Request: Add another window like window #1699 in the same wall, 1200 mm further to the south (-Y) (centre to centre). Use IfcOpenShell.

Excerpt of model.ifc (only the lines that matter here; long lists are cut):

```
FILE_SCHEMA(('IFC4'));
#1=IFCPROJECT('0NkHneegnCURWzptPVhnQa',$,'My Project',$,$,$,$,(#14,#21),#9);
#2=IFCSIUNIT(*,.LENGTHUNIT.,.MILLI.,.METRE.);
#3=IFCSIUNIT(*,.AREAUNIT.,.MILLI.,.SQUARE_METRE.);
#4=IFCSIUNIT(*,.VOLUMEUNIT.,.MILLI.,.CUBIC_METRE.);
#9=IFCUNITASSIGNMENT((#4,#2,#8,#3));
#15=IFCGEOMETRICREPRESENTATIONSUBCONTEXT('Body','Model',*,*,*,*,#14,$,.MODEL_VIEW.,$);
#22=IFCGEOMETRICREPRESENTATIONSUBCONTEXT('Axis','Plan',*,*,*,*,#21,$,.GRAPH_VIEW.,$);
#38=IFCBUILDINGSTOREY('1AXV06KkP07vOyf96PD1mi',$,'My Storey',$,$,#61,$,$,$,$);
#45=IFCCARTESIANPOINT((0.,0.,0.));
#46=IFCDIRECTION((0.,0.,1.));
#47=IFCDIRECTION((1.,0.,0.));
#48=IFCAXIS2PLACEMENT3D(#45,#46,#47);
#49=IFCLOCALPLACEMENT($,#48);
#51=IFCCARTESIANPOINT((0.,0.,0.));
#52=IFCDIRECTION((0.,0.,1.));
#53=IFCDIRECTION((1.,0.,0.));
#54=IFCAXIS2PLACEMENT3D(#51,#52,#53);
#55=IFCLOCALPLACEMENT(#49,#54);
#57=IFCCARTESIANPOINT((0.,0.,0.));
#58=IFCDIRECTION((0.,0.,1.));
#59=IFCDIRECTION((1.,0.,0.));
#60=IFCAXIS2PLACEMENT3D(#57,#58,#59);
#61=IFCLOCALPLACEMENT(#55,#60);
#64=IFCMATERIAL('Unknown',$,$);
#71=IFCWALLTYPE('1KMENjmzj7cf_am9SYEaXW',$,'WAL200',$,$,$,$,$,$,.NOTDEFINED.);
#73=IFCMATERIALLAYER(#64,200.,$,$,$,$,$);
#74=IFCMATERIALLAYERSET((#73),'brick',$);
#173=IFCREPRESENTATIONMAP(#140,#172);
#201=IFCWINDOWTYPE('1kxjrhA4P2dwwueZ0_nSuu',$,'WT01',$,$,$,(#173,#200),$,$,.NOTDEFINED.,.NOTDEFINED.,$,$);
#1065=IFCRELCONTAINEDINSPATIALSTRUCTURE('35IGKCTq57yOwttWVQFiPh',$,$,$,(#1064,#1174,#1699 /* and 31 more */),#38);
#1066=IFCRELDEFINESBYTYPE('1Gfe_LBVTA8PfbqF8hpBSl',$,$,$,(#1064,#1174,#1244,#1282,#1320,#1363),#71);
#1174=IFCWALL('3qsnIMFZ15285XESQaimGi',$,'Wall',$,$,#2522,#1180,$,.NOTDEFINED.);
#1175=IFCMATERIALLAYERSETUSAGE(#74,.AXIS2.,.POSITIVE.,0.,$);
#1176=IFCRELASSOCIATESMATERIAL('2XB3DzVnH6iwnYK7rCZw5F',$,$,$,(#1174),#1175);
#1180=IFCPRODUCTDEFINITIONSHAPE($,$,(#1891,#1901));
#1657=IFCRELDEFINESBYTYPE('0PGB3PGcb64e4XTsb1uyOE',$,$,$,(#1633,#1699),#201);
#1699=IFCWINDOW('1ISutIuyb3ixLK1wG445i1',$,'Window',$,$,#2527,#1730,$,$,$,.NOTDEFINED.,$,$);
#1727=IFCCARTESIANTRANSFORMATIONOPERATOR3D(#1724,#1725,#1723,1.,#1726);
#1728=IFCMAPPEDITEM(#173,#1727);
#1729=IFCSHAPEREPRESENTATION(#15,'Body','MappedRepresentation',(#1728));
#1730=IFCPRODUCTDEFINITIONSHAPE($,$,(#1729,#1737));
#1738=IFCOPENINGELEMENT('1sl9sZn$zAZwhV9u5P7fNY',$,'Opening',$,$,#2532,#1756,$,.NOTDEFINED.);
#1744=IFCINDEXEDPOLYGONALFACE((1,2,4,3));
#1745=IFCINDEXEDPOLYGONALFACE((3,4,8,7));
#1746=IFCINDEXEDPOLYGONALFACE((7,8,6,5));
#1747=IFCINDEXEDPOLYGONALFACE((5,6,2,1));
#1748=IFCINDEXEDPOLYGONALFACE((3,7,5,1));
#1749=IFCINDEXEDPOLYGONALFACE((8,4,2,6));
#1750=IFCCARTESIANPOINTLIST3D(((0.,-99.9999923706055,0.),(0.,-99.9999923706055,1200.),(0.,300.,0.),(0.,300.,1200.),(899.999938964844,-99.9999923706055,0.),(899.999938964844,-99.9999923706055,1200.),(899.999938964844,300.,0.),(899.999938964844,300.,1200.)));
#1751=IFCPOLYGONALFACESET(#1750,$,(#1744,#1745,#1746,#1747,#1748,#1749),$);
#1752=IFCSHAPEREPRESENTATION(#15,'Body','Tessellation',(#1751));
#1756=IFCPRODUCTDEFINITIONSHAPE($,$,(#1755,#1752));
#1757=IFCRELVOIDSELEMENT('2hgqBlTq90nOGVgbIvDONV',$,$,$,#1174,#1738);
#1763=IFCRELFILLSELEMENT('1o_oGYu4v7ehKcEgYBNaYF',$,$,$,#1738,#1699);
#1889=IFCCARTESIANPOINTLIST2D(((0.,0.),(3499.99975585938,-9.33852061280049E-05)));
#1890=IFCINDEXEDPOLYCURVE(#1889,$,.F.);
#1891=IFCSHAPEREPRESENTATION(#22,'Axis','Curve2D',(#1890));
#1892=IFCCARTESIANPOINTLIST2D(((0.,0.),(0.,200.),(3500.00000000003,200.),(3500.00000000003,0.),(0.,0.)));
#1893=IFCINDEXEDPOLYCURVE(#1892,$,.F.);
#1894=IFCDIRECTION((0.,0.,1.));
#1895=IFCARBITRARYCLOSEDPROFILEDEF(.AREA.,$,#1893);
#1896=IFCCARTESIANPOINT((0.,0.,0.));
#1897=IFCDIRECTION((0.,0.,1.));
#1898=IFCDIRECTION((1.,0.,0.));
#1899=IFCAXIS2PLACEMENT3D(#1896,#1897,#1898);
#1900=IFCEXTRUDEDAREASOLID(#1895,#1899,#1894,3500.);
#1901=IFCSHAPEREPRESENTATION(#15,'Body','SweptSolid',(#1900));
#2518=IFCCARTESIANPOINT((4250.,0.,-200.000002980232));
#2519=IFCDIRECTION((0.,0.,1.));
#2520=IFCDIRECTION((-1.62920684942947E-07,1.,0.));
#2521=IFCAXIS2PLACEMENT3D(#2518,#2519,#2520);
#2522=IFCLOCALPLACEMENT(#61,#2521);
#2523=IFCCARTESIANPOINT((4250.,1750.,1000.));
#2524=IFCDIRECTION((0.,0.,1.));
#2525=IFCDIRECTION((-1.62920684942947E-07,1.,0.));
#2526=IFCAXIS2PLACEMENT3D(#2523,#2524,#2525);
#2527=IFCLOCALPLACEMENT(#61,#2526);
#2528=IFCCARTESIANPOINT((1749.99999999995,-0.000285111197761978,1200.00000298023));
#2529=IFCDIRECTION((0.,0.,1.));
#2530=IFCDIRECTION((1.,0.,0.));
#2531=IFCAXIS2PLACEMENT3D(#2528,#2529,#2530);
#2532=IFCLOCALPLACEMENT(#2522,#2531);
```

```python
import ifcopenshell
import ifcopenshell.api.feature
import ifcopenshell.api.geometry
import ifcopenshell.api.root
import ifcopenshell.geom
import ifcopenshell.util.element
import ifcopenshell.util.placement
import ifcopenshell.util.shape
import ifcopenshell.util.unit

model = ifcopenshell.open("model.ifc")
unit_scale = ifcopenshell.util.unit.calculate_unit_scale(model)
settings = ifcopenshell.geom.settings()


def volume(element):
    """Net volume in cubic metres, openings subtracted."""
    shape = ifcopenshell.geom.create_shape(settings, element)
    return ifcopenshell.util.shape.get_volume(shape.geometry)


window = model.by_guid("1ISutIuyb3ixLK1wG445i1")
opening = window.FillsVoids[0].RelatingOpeningElement
wall = opening.VoidsElements[0].RelatingBuildingElement
before = volume(wall)
shift = ifcopenshell.util.placement.get_local_placement(wall.ObjectPlacement)[:3, 0] * -1.2 / unit_scale

# copy_class copies the void relationship, type, container and properties, but no geometry.
new_opening = ifcopenshell.api.root.copy_class(model, product=opening)
new_opening.Representation = ifcopenshell.util.element.copy_deep(
    model, opening.Representation, exclude=["IfcGeometricRepresentationContext", "IfcRepresentationMap"]
)
new_window = ifcopenshell.api.root.copy_class(model, product=window)
new_window.Representation = ifcopenshell.util.element.copy_deep(
    model, window.Representation, exclude=["IfcGeometricRepresentationContext", "IfcRepresentationMap"]
)
ifcopenshell.api.feature.add_filling(model, opening=new_opening, element=new_window)

for old, new in ((opening, new_opening), (window, new_window)):
    matrix = ifcopenshell.util.placement.get_local_placement(old.ObjectPlacement)
    matrix[:3, 3] += shift
    ifcopenshell.api.geometry.edit_object_placement(model, product=new, matrix=matrix, is_si=False)

after = volume(wall)

print(f"wall volume {before:.3f} -> {after:.3f} m3")

model.write("model_edited.ifc")
```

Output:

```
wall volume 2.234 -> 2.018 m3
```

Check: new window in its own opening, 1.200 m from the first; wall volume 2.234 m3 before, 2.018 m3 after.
